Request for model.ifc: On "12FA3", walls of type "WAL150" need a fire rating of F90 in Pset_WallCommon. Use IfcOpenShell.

First a look at what the model holds.

```python
import ifcopenshell
import ifcopenshell.util.element

model = ifcopenshell.open("model.ifc")
print(model.schema)
storey = next(s for s in model.by_type("IfcBuildingStorey") if s.Name == "12FA3")
walls = [e for e in ifcopenshell.util.element.get_decomposition(storey) if e.is_a("IfcWall")]
seen = {}
for e in walls:
    element_type = ifcopenshell.util.element.get_type(e)
    key = (element_type.Name if element_type != e and element_type else None, ifcopenshell.util.element.get_pset(e, "Pset_WallCommon", "FireRating"))
    seen[key] = seen.get(key, 0) + 1
for (name, value), count in sorted(seen.items(), key=str):
    print(count, "x", name, "|", value)
```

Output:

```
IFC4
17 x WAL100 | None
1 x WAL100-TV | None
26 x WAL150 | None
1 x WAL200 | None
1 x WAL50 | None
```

```python
import ifcopenshell
import ifcopenshell.api.pset
import ifcopenshell.util.element

model = ifcopenshell.open("model.ifc")

storey = next(s for s in model.by_type("IfcBuildingStorey") if s.Name == "12FA3")
walls = [e for e in ifcopenshell.util.element.get_decomposition(storey) if e.is_a("IfcWall")]

count = 0
for e in walls:
    element_type = ifcopenshell.util.element.get_type(e)
    if element_type in (None, e) or element_type.Name != "WAL150":
        continue
    # add_pset returns the element's existing set when there is one.
    pset = ifcopenshell.api.pset.add_pset(model, product=e, name="Pset_WallCommon")
    ifcopenshell.api.pset.edit_pset(model, pset=pset, properties={"FireRating": "F90"})
    count += 1

print(count, "walls updated")

model.write("model_edited.ifc")
```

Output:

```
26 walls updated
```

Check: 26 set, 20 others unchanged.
